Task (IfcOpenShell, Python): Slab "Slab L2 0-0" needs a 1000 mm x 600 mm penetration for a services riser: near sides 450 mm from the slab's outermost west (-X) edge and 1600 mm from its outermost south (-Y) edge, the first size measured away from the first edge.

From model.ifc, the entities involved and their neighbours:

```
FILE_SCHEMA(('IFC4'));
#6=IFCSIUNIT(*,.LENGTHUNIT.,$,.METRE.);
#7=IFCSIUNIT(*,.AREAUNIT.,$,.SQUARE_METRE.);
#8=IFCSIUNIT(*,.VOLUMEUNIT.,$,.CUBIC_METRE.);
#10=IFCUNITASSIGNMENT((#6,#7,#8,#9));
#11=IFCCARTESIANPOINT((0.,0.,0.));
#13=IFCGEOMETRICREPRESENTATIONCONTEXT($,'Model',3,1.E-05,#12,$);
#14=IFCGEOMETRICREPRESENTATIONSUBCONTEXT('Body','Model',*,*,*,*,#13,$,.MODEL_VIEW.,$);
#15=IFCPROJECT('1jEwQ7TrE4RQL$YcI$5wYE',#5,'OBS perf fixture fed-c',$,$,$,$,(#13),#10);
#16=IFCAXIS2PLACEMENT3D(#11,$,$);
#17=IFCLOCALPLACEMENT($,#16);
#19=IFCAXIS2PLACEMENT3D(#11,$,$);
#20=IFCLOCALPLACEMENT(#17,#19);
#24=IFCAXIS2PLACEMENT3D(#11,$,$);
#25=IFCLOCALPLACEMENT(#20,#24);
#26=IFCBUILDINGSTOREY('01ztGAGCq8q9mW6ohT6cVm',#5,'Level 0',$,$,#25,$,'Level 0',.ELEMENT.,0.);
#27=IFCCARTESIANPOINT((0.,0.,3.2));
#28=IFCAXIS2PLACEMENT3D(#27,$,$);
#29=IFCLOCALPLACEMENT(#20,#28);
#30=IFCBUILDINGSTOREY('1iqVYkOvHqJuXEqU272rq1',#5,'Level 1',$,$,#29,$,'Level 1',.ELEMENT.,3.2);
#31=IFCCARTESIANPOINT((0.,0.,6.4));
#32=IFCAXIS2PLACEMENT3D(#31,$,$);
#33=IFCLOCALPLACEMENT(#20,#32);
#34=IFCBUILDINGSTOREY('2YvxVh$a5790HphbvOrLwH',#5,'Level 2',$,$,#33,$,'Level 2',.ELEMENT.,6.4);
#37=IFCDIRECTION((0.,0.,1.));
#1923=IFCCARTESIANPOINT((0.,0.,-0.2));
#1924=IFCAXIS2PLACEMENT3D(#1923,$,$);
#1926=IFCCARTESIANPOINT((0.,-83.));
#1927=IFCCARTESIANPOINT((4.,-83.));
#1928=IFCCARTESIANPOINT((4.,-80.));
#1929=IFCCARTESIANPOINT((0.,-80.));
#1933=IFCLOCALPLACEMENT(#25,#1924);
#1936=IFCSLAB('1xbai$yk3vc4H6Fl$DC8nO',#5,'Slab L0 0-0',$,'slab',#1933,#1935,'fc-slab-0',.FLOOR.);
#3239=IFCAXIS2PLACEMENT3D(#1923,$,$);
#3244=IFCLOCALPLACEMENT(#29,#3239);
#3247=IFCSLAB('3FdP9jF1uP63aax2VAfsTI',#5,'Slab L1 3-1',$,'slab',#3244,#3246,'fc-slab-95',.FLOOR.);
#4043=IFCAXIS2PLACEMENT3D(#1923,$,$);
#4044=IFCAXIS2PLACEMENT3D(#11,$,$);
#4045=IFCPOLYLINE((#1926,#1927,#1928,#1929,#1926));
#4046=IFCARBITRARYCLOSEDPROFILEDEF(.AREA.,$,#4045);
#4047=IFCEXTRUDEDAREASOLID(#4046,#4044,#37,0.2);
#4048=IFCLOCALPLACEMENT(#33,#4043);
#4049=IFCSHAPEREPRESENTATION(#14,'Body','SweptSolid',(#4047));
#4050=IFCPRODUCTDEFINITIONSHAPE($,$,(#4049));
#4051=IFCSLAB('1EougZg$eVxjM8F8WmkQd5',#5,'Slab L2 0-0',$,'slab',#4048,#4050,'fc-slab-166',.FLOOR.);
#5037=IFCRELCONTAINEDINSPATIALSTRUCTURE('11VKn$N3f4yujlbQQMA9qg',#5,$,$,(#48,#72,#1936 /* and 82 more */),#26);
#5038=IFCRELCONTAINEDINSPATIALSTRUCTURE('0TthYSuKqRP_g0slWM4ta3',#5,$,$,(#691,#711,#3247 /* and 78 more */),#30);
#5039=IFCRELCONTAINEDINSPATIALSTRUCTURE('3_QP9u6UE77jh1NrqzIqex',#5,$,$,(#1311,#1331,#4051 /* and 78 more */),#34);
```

```python
import numpy as np
import ifcopenshell
import ifcopenshell.api.feature
import ifcopenshell.api.geometry
import ifcopenshell.api.root
import ifcopenshell.geom
import ifcopenshell.util.placement
import ifcopenshell.util.representation
import ifcopenshell.util.shape
import ifcopenshell.util.unit

model = ifcopenshell.open("model.ifc")
unit_scale = ifcopenshell.util.unit.calculate_unit_scale(model)
settings = ifcopenshell.geom.settings()


def volume(element):
    """Net volume in cubic metres, openings subtracted."""
    shape = ifcopenshell.geom.create_shape(settings, element)
    return ifcopenshell.util.shape.get_volume(shape.geometry)


slab = model.by_guid("1EougZg$eVxjM8F8WmkQd5")
before = volume(slab)

# Extent in the slab's own axes, in metres. The edges named are its -X and -Y sides.
slab_shape = ifcopenshell.geom.create_shape(settings, slab)
vertices = ifcopenshell.util.shape.get_vertices(slab_shape.geometry)
x_min, y_min, bottom = vertices.min(axis=0)
top = vertices[:, 2].max()

opening = ifcopenshell.api.root.create_entity(model, ifc_class="IfcOpeningElement", name="Services riser opening", predefined_type="OPENING")
context = ifcopenshell.util.representation.get_context(model, "Model", "Body", "MODEL_VIEW")
width, depth = 1, 0.6
outline = [(0.0, 0.0), (width, 0.0), (width, depth), (0.0, depth), (0.0, 0.0)]
# Overshoot both faces by 50 mm so the cut is clean.
shape = ifcopenshell.api.geometry.add_slab_representation(
    model, context=context, depth=top - bottom + 0.1, polyline=outline
)
ifcopenshell.api.geometry.assign_representation(model, product=opening, representation=shape)

matrix = ifcopenshell.util.placement.get_local_placement(slab.ObjectPlacement)
matrix[:, 3] = matrix @ np.append(np.array([x_min + 0.45, y_min + 1.6, bottom - 0.05]) / unit_scale, 1.0)
ifcopenshell.api.geometry.edit_object_placement(model, product=opening, matrix=matrix, is_si=False)
ifcopenshell.api.feature.add_feature(model, feature=opening, element=slab)

after = volume(slab)

print(f"slab volume {before:.3f} -> {after:.3f} m3")

model.write("model_updated.ifc")
```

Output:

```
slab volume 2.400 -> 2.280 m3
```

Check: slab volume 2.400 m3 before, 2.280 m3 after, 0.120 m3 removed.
